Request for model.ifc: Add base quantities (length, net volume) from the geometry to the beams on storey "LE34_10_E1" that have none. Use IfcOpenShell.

First a look at what the model holds.

```python
import ifcopenshell
import ifcopenshell.util.element
import ifcopenshell.util.unit

model = ifcopenshell.open("model.ifc")
print(model.schema)
for unit_type in ("LENGTHUNIT", "AREAUNIT", "VOLUMEUNIT"):
    print(unit_type, ifcopenshell.util.unit.calculate_unit_scale(model, unit_type))
storey = next(s for s in model.by_type("IfcBuildingStorey") if s.Name == "LE34_10_E1")
beams = [e for e in ifcopenshell.util.element.get_decomposition(storey) if e.is_a("IfcBeam")]
for e in sorted(beams, key=lambda e: e.id()):
    print(e.id(), e.is_a(), e.Name, list(ifcopenshell.util.element.get_psets(e, qtos_only=True)), sep=" | ")
```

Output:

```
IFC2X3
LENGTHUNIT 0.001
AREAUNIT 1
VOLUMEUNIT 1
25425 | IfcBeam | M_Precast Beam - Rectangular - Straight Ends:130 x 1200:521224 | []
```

```python
import ifcopenshell
import ifcopenshell.api.pset
import ifcopenshell.geom
import ifcopenshell.util.element
import ifcopenshell.util.shape
import ifcopenshell.util.unit

model = ifcopenshell.open("model.ifc")
unit_scale = ifcopenshell.util.unit.calculate_unit_scale(model)
volume_scale = ifcopenshell.util.unit.calculate_unit_scale(model, "VOLUMEUNIT")
settings = ifcopenshell.geom.settings()

storey = next(s for s in model.by_type("IfcBuildingStorey") if s.Name == "LE34_10_E1")
beams = [e for e in ifcopenshell.util.element.get_decomposition(storey) if e.is_a("IfcBeam")]

for e in sorted(beams, key=lambda e: e.id()):
    if ifcopenshell.util.element.get_psets(e, qtos_only=True, should_inherit=False):
        continue
    # Geometry comes back in metres, in the element's own axes.
    shape = ifcopenshell.geom.create_shape(settings, e)
    values = {
        "Length": ifcopenshell.util.shape.get_max_xyz(shape.geometry) / unit_scale,
        "NetVolume": ifcopenshell.util.shape.get_volume(shape.geometry) / volume_scale,
    }
    qto = ifcopenshell.api.pset.add_qto(model, product=e, name="BaseQuantities")
    ifcopenshell.api.pset.edit_qto(model, qto=qto, properties=values)
    print(e.id(), {k: round(v, 3) for k, v in values.items()})

model.write("model_edited.ifc")
```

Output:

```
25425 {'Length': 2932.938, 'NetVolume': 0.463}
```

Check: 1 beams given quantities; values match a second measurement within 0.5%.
